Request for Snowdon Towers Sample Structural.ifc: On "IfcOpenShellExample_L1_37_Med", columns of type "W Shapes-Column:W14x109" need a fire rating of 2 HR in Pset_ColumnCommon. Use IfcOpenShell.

First a look at what the model holds.

```python
import ifcopenshell
import ifcopenshell.util.element

model = ifcopenshell.open("Snowdon Towers Sample Structural.ifc")
print(model.schema)
storey = next(s for s in model.by_type("IfcBuildingStorey") if s.Name == "IfcOpenShellExample_L1_37_Med")
columns = [e for e in ifcopenshell.util.element.get_decomposition(storey) if e.is_a("IfcColumn")]
seen = {}
for e in columns:
    element_type = ifcopenshell.util.element.get_type(e)
    key = (element_type.Name if element_type != e and element_type else None, ifcopenshell.util.element.get_pset(e, "Pset_ColumnCommon", "FireRating"))
    seen[key] = seen.get(key, 0) + 1
for (name, value), count in sorted(seen.items(), key=str):
    print(count, "x", name, "|", value)
```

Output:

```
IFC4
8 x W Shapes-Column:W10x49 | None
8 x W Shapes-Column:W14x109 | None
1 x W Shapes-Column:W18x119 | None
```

```python
import ifcopenshell
import ifcopenshell.api.pset
import ifcopenshell.util.element

model = ifcopenshell.open("Snowdon Towers Sample Structural.ifc")

storey = next(s for s in model.by_type("IfcBuildingStorey") if s.Name == "IfcOpenShellExample_L1_37_Med")
columns = [e for e in ifcopenshell.util.element.get_decomposition(storey) if e.is_a("IfcColumn")]

count = 0
for e in columns:
    element_type = ifcopenshell.util.element.get_type(e)
    if element_type in (None, e) or element_type.Name != "W Shapes-Column:W14x109":
        continue
    # add_pset returns the element's existing set when there is one.
    pset = ifcopenshell.api.pset.add_pset(model, product=e, name="Pset_ColumnCommon")
    ifcopenshell.api.pset.edit_pset(model, pset=pset, properties={"FireRating": "2 HR"})
    count += 1

print(count, "columns updated")

model.write("Snowdon Towers Sample Structural_v2.ifc")
```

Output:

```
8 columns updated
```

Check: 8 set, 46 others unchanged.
